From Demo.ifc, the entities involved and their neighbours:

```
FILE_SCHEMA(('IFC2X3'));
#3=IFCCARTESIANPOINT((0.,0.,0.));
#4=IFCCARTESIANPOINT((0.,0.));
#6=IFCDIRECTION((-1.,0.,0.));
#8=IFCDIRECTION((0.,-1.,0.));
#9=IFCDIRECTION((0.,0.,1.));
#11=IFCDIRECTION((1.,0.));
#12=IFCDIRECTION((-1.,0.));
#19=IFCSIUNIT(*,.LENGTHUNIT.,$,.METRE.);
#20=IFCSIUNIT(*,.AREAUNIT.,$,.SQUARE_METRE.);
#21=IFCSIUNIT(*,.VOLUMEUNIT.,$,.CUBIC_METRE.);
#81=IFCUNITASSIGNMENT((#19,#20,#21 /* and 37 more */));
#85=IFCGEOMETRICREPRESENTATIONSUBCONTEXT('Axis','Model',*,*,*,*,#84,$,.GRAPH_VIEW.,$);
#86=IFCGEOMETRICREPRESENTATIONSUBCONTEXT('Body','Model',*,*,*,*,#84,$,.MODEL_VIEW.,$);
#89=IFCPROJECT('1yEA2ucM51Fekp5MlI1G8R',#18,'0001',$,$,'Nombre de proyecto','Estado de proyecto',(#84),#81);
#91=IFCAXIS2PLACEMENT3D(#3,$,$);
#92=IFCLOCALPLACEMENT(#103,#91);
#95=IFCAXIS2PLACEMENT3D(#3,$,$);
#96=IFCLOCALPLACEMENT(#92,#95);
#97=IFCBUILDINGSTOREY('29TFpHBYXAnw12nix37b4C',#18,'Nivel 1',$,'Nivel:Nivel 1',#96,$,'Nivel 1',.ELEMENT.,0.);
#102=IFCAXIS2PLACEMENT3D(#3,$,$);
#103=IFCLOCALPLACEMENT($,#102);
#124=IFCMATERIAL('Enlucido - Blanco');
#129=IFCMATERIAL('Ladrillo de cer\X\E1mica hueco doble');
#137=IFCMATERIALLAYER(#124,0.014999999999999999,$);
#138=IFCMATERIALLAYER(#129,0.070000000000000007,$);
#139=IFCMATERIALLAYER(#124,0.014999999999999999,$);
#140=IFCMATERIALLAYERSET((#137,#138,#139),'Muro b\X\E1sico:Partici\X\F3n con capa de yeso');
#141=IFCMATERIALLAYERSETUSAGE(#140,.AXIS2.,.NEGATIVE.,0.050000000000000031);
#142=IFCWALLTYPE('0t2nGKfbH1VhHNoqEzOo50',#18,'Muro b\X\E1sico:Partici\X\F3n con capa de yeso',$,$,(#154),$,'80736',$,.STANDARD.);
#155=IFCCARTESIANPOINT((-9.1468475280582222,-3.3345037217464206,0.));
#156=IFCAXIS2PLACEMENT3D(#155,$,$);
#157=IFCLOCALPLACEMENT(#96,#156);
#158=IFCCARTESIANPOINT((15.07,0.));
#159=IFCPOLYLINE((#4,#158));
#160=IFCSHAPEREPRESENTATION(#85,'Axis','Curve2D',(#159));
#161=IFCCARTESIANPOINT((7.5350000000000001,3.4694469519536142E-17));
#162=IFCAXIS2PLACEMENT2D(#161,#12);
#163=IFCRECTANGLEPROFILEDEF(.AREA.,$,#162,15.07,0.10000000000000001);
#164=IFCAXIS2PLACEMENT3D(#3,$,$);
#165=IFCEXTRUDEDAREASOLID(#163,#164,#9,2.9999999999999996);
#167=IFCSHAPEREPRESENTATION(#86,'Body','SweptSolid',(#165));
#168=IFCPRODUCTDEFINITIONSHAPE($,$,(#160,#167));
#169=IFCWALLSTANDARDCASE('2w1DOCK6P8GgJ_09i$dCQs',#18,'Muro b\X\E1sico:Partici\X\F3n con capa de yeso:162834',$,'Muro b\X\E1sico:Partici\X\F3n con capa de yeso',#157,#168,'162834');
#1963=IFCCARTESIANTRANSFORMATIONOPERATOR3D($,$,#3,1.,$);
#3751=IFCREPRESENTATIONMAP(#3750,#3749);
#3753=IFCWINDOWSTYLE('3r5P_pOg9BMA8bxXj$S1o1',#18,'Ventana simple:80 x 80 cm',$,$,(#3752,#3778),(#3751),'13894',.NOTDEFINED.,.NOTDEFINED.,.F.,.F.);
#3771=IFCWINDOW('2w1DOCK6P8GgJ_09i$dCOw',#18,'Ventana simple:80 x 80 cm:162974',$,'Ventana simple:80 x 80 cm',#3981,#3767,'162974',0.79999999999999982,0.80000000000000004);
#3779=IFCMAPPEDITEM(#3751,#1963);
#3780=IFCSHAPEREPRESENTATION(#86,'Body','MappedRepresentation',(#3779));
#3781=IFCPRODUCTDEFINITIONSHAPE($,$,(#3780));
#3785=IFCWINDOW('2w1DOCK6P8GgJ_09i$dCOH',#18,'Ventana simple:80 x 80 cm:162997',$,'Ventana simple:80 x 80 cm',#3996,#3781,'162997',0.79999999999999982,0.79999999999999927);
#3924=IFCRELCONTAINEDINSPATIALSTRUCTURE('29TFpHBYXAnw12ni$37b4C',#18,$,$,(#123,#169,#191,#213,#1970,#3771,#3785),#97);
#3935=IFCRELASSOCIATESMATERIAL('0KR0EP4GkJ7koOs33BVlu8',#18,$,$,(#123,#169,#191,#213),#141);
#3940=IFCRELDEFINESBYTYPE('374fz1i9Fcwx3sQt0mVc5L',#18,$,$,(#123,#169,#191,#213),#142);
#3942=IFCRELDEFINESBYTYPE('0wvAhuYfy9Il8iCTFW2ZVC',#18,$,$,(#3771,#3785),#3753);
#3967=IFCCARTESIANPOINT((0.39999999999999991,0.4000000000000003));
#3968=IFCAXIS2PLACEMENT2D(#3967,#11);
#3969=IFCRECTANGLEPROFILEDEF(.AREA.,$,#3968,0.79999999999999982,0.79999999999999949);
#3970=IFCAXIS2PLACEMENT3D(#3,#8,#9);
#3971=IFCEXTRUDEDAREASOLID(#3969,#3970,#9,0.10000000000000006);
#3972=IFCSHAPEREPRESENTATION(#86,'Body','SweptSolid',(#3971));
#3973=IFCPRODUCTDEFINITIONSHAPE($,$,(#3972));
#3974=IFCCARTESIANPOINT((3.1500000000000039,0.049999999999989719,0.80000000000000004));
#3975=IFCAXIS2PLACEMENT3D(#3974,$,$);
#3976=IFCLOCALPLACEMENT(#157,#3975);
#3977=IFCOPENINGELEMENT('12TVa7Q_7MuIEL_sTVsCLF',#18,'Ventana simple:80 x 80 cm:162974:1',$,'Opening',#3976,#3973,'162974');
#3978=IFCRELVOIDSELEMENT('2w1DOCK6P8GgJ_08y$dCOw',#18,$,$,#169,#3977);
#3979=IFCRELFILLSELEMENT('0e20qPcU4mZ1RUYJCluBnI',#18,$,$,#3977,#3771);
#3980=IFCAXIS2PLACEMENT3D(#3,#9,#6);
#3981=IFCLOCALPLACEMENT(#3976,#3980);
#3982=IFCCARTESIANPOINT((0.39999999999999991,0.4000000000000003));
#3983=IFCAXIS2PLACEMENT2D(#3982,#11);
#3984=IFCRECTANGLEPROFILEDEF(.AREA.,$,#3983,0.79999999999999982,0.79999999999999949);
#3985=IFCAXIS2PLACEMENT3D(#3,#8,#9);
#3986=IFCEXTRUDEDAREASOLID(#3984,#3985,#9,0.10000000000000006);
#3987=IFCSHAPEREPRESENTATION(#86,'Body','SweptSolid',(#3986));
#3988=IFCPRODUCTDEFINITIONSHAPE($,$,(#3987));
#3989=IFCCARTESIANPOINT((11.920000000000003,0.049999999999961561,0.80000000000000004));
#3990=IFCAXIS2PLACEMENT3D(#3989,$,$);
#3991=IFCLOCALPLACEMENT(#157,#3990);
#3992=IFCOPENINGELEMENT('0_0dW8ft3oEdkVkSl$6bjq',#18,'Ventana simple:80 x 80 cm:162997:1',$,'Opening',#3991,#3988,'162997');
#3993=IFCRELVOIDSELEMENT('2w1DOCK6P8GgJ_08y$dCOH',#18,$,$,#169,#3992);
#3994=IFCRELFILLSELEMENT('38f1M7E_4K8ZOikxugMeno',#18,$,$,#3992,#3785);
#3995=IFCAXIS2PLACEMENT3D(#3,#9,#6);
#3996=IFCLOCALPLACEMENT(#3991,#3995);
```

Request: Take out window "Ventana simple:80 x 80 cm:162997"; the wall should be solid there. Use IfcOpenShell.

```python
import ifcopenshell
import ifcopenshell.api.feature
import ifcopenshell.api.root
import ifcopenshell.geom
import ifcopenshell.util.shape

model = ifcopenshell.open("Demo.ifc")
settings = ifcopenshell.geom.settings()


def volume(element):
    """Net volume in cubic metres, openings subtracted."""
    shape = ifcopenshell.geom.create_shape(settings, element)
    return ifcopenshell.util.shape.get_volume(shape.geometry)


window = model.by_guid("2w1DOCK6P8GgJ_09i$dCOH")
opening = window.FillsVoids[0].RelatingOpeningElement
wall = opening.VoidsElements[0].RelatingBuildingElement
before = volume(wall)

ifcopenshell.api.root.remove_product(model, product=window)
ifcopenshell.api.feature.remove_feature(model, feature=opening)

after = volume(wall)

print(f"wall volume {before:.3f} -> {after:.3f} m3")

model.write("Demo_rev.ifc")
```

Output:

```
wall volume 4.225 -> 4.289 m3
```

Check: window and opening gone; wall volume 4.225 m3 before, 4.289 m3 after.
